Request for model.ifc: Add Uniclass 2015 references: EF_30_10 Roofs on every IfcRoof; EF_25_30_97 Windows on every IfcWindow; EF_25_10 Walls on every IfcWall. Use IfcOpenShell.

First a look at what the model holds.

```python
import ifcopenshell

model = ifcopenshell.open("model.ifc")
print(model.schema)
print("classifications:", [c.Name for c in model.by_type("IfcClassification")])
for ifc_class in ("IfcDoor", "IfcRoof", "IfcStair", "IfcWall", "IfcWindow"):
    print(ifc_class, len(model.by_type(ifc_class)))
```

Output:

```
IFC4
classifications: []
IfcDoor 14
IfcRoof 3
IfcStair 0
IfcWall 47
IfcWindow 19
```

```python
import ifcopenshell
import ifcopenshell.api.classification

model = ifcopenshell.open("model.ifc")

system = ifcopenshell.api.classification.add_classification(model, classification="Uniclass 2015")

codes = {
    "IfcRoof": ("EF_30_10", "Roofs"),
    "IfcWindow": ("EF_25_30_97", "Windows"),
    "IfcWall": ("EF_25_10", "Walls"),
}
for ifc_class, (code, name) in codes.items():
    products = model.by_type(ifc_class)
    ifcopenshell.api.classification.add_reference(
        model, products=products, classification=system, identification=code, name=name
    )
    print(code, len(products))

model.write("model_updated.ifc")
```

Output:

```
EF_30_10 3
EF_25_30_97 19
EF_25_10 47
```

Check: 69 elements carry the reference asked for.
